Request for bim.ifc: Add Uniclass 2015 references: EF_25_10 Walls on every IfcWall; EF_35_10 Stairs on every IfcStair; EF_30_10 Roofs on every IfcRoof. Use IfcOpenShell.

First a look at what the model holds.

```python
import ifcopenshell

model = ifcopenshell.open("bim.ifc")
print(model.schema)
print("classifications:", [c.Name for c in model.by_type("IfcClassification")])
for ifc_class in ("IfcDoor", "IfcRoof", "IfcStair", "IfcWall", "IfcWindow"):
    print(ifc_class, len(model.by_type(ifc_class)))
```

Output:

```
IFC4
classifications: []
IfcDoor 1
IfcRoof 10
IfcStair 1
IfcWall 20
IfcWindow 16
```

```python
import ifcopenshell
import ifcopenshell.api.classification

model = ifcopenshell.open("bim.ifc")

system = ifcopenshell.api.classification.add_classification(model, classification="Uniclass 2015")

codes = {
    "IfcWall": ("EF_25_10", "Walls"),
    "IfcStair": ("EF_35_10", "Stairs"),
    "IfcRoof": ("EF_30_10", "Roofs"),
}
for ifc_class, (code, name) in codes.items():
    products = model.by_type(ifc_class)
    ifcopenshell.api.classification.add_reference(
        model, products=products, classification=system, identification=code, name=name
    )
    print(code, len(products))

model.write("bim_v2.ifc")
```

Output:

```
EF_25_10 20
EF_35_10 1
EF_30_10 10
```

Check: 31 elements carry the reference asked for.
